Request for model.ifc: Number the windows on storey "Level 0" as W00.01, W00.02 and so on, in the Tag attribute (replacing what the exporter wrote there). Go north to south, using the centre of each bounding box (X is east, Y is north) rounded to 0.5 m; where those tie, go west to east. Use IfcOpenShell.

First a look at what the model holds.

```python
import ifcopenshell
import ifcopenshell.util.element
import ifcopenshell.util.placement

model = ifcopenshell.open("model.ifc")
print(model.schema)
storey = next(s for s in model.by_type("IfcBuildingStorey") if s.Name == "Level 0")
windows = [e for e in ifcopenshell.util.element.get_decomposition(storey) if e.is_a("IfcWindow")]
for e in sorted(windows, key=lambda e: e.id()):
    origin = ifcopenshell.util.placement.get_local_placement(e.ObjectPlacement)[:3, 3]
    print(e.id(), e.Tag, e.Name, origin.round(2) + 0.0, sep=" | ")
```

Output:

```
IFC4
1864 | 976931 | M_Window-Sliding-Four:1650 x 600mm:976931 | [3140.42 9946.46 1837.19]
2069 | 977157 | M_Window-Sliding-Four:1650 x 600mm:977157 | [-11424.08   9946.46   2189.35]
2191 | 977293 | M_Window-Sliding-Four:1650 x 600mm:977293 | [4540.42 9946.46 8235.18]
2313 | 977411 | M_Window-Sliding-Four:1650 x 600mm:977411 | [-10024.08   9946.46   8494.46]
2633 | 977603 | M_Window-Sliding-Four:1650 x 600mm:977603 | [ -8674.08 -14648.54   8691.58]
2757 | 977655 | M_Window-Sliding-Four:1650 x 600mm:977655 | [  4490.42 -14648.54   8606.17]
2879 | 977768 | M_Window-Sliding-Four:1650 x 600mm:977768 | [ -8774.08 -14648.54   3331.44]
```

```python
import ifcopenshell
import ifcopenshell.geom
import ifcopenshell.util.element
import ifcopenshell.util.shape

model = ifcopenshell.open("model.ifc")
settings = ifcopenshell.geom.settings()
settings.set("use-world-coords", True)


def centre(element):
    shape = ifcopenshell.geom.create_shape(settings, element)
    return ifcopenshell.util.shape.get_bbox_centroid(shape.geometry)


storey = next(s for s in model.by_type("IfcBuildingStorey") if s.Name == "Level 0")
windows = [e for e in ifcopenshell.util.element.get_decomposition(storey) if e.is_a("IfcWindow")]

# Insertion points can sit at a corner or the storey origin, so sort by the geometry (in metres).
centres = {e: centre(e) for e in windows}
windows.sort(key=lambda e: (-round(centres[e][1] / 0.5), centres[e][0]))

for i, e in enumerate(windows, start=1):
    number = f"W00.{i:02d}"
    e.Tag = number
    print(e.id(), number)

model.write("model-out.ifc")
```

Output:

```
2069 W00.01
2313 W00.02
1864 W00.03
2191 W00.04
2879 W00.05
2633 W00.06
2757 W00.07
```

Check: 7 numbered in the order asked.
